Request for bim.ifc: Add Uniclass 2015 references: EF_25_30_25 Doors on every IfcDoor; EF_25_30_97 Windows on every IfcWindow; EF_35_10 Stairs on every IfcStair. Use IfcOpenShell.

First a look at what the model holds.

```python
import ifcopenshell

model = ifcopenshell.open("bim.ifc")
print(model.schema)
print("classifications:", [c.Name for c in model.by_type("IfcClassification")])
for ifc_class in ("IfcDoor", "IfcRoof", "IfcStair", "IfcWall", "IfcWindow"):
    print(ifc_class, len(model.by_type(ifc_class)))
```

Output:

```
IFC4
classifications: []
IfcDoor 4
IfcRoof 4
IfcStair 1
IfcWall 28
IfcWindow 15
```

```python
import ifcopenshell
import ifcopenshell.api.classification

model = ifcopenshell.open("bim.ifc")

system = ifcopenshell.api.classification.add_classification(model, classification="Uniclass 2015")

codes = {
    "IfcDoor": ("EF_25_30_25", "Doors"),
    "IfcWindow": ("EF_25_30_97", "Windows"),
    "IfcStair": ("EF_35_10", "Stairs"),
}
for ifc_class, (code, name) in codes.items():
    products = model.by_type(ifc_class)
    ifcopenshell.api.classification.add_reference(
        model, products=products, classification=system, identification=code, name=name
    )
    print(code, len(products))

model.write("bim_updated.ifc")
```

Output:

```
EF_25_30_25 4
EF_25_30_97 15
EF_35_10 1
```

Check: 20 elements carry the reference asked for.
